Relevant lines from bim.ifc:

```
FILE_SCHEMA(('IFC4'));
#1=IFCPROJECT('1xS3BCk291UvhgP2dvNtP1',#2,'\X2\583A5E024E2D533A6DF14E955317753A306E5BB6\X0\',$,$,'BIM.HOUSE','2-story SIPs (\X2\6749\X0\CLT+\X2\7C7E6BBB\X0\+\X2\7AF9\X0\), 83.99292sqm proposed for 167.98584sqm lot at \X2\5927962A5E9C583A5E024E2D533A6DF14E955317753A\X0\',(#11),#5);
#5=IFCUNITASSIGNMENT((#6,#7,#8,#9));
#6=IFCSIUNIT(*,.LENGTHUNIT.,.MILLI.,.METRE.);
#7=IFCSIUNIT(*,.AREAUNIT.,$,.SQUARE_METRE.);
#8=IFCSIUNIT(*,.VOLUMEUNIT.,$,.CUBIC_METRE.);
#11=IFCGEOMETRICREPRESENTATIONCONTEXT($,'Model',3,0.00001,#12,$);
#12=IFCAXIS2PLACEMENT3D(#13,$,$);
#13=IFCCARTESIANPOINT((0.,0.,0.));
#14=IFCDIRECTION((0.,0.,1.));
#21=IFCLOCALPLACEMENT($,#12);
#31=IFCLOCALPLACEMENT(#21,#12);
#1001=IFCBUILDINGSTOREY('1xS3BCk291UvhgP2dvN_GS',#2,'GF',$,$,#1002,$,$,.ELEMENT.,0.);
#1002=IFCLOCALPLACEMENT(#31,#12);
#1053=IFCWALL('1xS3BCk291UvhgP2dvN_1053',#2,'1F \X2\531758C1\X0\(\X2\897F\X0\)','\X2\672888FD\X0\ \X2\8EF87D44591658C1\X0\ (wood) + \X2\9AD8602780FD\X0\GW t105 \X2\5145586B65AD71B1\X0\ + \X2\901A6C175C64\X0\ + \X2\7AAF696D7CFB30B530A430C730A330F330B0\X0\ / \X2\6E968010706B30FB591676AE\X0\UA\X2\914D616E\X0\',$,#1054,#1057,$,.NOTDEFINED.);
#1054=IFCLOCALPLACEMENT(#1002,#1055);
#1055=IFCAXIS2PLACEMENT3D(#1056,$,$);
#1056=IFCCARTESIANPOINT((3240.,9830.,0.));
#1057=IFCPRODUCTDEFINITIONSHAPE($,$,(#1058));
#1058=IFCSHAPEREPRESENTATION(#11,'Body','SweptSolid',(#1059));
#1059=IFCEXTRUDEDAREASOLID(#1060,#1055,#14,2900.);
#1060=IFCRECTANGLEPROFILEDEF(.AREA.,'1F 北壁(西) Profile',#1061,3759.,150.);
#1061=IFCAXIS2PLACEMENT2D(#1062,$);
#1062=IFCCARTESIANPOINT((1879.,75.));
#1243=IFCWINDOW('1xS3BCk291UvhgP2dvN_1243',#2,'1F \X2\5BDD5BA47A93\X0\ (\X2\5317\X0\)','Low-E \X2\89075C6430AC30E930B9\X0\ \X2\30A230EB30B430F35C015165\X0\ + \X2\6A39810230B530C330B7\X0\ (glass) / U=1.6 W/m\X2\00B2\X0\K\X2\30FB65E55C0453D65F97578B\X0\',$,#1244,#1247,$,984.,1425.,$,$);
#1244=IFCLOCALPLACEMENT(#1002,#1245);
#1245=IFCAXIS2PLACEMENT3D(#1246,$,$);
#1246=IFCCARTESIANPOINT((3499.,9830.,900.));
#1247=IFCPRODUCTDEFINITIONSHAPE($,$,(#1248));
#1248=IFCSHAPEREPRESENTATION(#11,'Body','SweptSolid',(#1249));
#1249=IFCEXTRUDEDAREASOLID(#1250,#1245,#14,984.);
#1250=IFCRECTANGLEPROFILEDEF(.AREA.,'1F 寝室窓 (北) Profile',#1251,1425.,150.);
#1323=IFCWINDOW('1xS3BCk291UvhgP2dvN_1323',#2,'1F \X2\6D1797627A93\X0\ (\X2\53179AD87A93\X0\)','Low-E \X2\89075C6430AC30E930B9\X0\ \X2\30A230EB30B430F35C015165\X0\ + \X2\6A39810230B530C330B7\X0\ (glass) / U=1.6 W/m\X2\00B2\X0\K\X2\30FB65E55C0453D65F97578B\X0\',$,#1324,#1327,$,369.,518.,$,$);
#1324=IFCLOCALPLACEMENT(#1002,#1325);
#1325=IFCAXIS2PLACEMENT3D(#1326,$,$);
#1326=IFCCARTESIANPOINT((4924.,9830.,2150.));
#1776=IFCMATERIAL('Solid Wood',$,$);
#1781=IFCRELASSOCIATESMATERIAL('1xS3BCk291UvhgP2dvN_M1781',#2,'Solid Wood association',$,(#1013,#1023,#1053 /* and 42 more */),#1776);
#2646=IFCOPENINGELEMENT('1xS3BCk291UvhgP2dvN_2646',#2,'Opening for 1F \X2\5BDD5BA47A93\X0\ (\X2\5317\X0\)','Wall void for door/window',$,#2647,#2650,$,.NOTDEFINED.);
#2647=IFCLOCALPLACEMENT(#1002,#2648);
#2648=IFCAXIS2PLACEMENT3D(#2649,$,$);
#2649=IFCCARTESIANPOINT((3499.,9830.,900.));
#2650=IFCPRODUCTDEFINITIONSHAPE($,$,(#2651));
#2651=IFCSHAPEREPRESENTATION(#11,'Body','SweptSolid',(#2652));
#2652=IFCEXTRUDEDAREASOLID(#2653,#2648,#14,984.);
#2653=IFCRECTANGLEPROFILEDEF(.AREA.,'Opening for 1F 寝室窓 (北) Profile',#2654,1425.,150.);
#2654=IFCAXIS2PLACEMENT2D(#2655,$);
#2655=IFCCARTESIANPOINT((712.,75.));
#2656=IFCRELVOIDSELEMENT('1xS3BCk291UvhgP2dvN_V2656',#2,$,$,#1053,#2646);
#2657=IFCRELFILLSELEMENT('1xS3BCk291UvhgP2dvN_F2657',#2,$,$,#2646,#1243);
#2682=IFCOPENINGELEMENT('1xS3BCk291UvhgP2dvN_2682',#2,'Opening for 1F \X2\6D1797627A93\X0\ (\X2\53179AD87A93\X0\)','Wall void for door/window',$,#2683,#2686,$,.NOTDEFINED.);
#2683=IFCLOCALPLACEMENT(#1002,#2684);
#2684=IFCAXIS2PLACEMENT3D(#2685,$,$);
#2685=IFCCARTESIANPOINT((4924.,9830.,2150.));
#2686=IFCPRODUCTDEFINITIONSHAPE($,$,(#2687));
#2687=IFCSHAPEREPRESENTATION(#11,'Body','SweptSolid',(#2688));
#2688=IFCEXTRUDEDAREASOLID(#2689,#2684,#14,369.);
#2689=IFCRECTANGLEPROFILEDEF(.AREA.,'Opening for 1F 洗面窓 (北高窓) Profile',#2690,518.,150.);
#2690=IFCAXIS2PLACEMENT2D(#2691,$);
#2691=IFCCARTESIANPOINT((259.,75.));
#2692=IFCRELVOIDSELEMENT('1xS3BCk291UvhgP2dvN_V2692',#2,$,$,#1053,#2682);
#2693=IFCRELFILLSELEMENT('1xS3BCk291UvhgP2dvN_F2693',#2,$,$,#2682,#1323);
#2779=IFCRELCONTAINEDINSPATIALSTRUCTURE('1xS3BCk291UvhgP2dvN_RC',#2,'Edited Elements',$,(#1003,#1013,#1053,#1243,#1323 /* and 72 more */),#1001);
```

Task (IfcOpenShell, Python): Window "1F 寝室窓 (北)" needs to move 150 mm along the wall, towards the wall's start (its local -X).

```python
import ifcopenshell
import ifcopenshell.api.geometry
import ifcopenshell.util.placement

model = ifcopenshell.open("bim.ifc")

window = model.by_guid("1xS3BCk291UvhgP2dvN_1243")
opening = window.FillsVoids[0].RelatingOpeningElement
wall = opening.VoidsElements[0].RelatingBuildingElement

wall_matrix = ifcopenshell.util.placement.get_local_placement(wall.ObjectPlacement)
shift = wall_matrix[:3, 0] * -150.0
before = ifcopenshell.util.placement.get_local_placement(window.ObjectPlacement)[:3, 3].copy()

# The window is not placed relative to its opening, so move both.
for product in (opening, window):
    matrix = ifcopenshell.util.placement.get_local_placement(product.ObjectPlacement)
    matrix[:3, 3] += shift
    ifcopenshell.api.geometry.edit_object_placement(model, product=product, matrix=matrix, is_si=False)

after = ifcopenshell.util.placement.get_local_placement(window.ObjectPlacement)[:3, 3]
print("window moved by", (after - before).round(3) + 0.0)

model.write("bim_v2.ifc")
```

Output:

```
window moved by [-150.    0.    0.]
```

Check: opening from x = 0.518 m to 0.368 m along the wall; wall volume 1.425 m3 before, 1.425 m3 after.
